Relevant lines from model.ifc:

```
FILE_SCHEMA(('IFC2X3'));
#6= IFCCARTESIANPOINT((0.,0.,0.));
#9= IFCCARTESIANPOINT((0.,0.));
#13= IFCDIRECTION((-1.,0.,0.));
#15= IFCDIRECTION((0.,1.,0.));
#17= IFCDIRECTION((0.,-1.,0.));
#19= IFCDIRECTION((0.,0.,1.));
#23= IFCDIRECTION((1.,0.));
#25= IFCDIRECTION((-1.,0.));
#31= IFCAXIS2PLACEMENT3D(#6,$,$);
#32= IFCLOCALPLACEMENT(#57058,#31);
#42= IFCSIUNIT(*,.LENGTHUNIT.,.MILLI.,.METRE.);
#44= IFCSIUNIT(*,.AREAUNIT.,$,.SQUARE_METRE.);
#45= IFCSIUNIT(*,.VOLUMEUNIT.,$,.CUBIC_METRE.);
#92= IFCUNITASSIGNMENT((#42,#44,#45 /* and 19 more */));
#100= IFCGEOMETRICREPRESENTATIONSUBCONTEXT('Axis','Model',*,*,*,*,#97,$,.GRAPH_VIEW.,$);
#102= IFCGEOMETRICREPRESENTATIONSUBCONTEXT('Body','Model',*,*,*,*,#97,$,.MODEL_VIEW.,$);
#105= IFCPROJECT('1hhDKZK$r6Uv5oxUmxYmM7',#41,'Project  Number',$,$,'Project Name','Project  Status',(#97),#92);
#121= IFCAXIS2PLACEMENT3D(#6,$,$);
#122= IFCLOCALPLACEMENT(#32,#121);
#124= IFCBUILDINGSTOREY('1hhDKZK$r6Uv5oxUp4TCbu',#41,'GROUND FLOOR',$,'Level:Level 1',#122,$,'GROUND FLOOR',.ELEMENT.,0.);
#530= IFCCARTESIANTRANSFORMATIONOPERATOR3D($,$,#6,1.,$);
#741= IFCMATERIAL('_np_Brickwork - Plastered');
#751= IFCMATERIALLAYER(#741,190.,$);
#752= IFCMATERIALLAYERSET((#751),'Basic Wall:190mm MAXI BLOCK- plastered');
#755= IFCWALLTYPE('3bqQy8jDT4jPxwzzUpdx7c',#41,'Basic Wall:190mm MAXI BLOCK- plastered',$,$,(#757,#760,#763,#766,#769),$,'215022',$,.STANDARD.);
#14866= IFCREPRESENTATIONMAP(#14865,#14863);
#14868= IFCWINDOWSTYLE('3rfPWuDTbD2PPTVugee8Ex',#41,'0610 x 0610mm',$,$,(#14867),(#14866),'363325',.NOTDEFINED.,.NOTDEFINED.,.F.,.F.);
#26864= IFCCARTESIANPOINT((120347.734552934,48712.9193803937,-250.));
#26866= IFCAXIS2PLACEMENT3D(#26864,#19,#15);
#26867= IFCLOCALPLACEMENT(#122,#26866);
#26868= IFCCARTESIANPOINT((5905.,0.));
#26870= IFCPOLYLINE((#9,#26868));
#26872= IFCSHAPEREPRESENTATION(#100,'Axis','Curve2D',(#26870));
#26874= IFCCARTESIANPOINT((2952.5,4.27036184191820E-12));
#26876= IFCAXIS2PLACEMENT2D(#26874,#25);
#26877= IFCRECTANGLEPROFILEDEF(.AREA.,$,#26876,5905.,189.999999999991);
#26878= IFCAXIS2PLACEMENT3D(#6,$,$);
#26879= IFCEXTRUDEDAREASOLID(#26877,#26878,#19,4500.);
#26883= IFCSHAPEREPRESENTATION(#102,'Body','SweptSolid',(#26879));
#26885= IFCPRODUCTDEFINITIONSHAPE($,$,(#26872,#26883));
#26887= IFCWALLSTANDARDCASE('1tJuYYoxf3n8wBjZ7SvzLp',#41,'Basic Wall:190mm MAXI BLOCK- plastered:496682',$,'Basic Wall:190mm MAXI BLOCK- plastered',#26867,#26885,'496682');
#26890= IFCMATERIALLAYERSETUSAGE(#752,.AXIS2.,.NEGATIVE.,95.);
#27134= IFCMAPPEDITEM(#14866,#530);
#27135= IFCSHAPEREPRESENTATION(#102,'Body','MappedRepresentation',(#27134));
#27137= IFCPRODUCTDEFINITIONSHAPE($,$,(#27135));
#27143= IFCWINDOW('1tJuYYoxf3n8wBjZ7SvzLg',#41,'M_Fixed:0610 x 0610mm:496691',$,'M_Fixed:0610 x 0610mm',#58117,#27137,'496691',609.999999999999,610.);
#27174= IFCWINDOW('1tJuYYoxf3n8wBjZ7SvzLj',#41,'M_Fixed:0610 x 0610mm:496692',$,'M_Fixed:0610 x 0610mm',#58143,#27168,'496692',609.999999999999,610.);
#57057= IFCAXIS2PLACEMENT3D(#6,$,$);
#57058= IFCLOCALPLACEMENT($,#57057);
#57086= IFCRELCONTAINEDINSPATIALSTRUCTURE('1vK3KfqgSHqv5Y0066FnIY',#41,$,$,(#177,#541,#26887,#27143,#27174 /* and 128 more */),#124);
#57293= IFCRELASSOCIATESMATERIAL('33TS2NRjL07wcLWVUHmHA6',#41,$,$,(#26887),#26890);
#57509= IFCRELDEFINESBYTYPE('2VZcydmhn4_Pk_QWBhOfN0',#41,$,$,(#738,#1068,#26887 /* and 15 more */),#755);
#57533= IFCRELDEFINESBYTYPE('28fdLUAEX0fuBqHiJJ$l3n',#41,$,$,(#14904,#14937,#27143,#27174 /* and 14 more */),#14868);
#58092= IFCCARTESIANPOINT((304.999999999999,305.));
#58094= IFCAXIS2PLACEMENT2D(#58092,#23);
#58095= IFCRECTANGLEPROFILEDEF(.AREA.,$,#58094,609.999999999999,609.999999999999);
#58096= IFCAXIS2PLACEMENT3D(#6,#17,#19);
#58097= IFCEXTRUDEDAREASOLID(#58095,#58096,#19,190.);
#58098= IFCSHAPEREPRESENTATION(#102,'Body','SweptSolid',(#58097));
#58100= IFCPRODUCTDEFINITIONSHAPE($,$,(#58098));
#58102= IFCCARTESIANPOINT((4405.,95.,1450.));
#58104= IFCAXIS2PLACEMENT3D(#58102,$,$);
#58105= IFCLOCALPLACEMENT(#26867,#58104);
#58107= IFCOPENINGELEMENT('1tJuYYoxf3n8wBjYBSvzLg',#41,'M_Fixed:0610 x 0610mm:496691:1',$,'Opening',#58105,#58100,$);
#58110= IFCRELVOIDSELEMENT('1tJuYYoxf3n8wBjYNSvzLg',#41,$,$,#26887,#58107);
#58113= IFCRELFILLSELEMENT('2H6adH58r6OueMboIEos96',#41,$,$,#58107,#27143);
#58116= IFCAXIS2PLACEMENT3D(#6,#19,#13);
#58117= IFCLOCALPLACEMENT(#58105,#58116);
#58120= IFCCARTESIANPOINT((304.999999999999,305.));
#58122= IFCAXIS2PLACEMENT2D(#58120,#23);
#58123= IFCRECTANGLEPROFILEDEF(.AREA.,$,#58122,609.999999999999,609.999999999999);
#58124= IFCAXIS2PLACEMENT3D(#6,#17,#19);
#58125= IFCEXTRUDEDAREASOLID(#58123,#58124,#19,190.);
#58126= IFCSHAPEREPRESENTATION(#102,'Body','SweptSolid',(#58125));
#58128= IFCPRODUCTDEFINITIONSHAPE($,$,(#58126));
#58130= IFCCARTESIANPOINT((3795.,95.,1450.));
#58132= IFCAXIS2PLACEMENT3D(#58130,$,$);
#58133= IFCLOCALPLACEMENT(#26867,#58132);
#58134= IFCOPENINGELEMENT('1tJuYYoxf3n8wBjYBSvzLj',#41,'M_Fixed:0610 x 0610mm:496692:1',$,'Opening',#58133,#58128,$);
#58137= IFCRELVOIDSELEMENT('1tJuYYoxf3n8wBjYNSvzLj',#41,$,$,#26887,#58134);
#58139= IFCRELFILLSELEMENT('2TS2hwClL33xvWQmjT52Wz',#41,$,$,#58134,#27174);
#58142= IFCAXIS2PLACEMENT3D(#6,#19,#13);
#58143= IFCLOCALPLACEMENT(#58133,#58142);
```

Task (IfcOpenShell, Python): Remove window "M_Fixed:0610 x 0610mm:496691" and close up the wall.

```python
import ifcopenshell
import ifcopenshell.api.feature
import ifcopenshell.api.root
import ifcopenshell.geom
import ifcopenshell.util.shape

model = ifcopenshell.open("model.ifc")
settings = ifcopenshell.geom.settings()


def volume(element):
    """Net volume in cubic metres, openings subtracted."""
    shape = ifcopenshell.geom.create_shape(settings, element)
    return ifcopenshell.util.shape.get_volume(shape.geometry)


window = model.by_id(27143)
opening = window.FillsVoids[0].RelatingOpeningElement
wall = opening.VoidsElements[0].RelatingBuildingElement
before = volume(wall)

ifcopenshell.api.root.remove_product(model, product=window)
ifcopenshell.api.feature.remove_feature(model, feature=opening)

after = volume(wall)

print(f"wall volume {before:.3f} -> {after:.3f} m3")

model.write("model_rev.ifc")
```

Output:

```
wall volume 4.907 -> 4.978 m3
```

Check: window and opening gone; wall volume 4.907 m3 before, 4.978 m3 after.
